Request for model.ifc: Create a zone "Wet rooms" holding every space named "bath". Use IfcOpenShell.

First a look at what the model holds.

```python
import ifcopenshell

model = ifcopenshell.open("model.ifc")
print(model.schema)
seen = {}
for space in model.by_type("IfcSpace"):
    seen[space.LongName] = seen.get(space.LongName, 0) + 1
for name, count in sorted(seen.items(), key=str):
    print(count, "x", name)
print("zones:", [z.Name for z in model.by_type("IfcZone")][:20])
```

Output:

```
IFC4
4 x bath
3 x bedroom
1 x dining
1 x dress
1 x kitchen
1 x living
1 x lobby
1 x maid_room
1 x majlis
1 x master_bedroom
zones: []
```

```python
import ifcopenshell
import ifcopenshell.api.group
import ifcopenshell.api.root

model = ifcopenshell.open("model.ifc")

names = {"bath"}
spaces = [s for s in model.by_type("IfcSpace") if s.LongName in names]

zone = ifcopenshell.api.root.create_entity(model, ifc_class="IfcZone", name="Wet rooms")
ifcopenshell.api.group.assign_group(model, products=spaces, group=zone)
print(len(spaces), "spaces in", zone.Name)

model.write("model_edited.ifc")
```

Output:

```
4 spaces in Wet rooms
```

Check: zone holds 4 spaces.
